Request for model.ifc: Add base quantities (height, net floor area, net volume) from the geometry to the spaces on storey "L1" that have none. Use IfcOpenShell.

First a look at what the model holds.

```python
import ifcopenshell
import ifcopenshell.util.element
import ifcopenshell.util.unit

model = ifcopenshell.open("model.ifc")
print(model.schema)
for unit_type in ("LENGTHUNIT", "AREAUNIT", "VOLUMEUNIT"):
    print(unit_type, ifcopenshell.util.unit.calculate_unit_scale(model, unit_type))
storey = next(s for s in model.by_type("IfcBuildingStorey") if s.Name == "L1")
spaces = [e for e in ifcopenshell.util.element.get_decomposition(storey) if e.is_a("IfcSpace")]
for e in sorted(spaces, key=lambda e: e.id()):
    print(e.id(), e.is_a(), e.Name, list(ifcopenshell.util.element.get_psets(e, qtos_only=True)), sep=" | ")
```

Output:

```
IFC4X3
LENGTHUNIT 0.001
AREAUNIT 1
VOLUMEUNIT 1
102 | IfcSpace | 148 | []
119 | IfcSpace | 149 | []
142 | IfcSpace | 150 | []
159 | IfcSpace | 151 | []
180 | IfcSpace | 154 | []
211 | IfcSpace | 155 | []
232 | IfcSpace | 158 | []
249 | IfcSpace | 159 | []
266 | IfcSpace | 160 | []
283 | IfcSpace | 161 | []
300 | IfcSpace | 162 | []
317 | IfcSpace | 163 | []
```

```python
import ifcopenshell
import ifcopenshell.api.pset
import ifcopenshell.geom
import ifcopenshell.util.element
import ifcopenshell.util.shape
import ifcopenshell.util.unit

model = ifcopenshell.open("model.ifc")
unit_scale = ifcopenshell.util.unit.calculate_unit_scale(model)
area_scale = ifcopenshell.util.unit.calculate_unit_scale(model, "AREAUNIT")
volume_scale = ifcopenshell.util.unit.calculate_unit_scale(model, "VOLUMEUNIT")
settings = ifcopenshell.geom.settings()

storey = next(s for s in model.by_type("IfcBuildingStorey") if s.Name == "L1")
spaces = [e for e in ifcopenshell.util.element.get_decomposition(storey) if e.is_a("IfcSpace")]

for e in sorted(spaces, key=lambda e: e.id()):
    if ifcopenshell.util.element.get_psets(e, qtos_only=True, should_inherit=False):
        continue
    # Geometry comes back in metres, in the element's own axes.
    shape = ifcopenshell.geom.create_shape(settings, e)
    values = {
        "Height": ifcopenshell.util.shape.get_z(shape.geometry) / unit_scale,
        "NetFloorArea": ifcopenshell.util.shape.get_footprint_area(shape.geometry) / area_scale,
        "NetVolume": ifcopenshell.util.shape.get_volume(shape.geometry) / volume_scale,
    }
    qto = ifcopenshell.api.pset.add_qto(model, product=e, name="Qto_SpaceBaseQuantities")
    ifcopenshell.api.pset.edit_qto(model, qto=qto, properties=values)
    print(e.id(), {k: round(v, 3) for k, v in values.items()})

model.write("model_rev.ifc")
```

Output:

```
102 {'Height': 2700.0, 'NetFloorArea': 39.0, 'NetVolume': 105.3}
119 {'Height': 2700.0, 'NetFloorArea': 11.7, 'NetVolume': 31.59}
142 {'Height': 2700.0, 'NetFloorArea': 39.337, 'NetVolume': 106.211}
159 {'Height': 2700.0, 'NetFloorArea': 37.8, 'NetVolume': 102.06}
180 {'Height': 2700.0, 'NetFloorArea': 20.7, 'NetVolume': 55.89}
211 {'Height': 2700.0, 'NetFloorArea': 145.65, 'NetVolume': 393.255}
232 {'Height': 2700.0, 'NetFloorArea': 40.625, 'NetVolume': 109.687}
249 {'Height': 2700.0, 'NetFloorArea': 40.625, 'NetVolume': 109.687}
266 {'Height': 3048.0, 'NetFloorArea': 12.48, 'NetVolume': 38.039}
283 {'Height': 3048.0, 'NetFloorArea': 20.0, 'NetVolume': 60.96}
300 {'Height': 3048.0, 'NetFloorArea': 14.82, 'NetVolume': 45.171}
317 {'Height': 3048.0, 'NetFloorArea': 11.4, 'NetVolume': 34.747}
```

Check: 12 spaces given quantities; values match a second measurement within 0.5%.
